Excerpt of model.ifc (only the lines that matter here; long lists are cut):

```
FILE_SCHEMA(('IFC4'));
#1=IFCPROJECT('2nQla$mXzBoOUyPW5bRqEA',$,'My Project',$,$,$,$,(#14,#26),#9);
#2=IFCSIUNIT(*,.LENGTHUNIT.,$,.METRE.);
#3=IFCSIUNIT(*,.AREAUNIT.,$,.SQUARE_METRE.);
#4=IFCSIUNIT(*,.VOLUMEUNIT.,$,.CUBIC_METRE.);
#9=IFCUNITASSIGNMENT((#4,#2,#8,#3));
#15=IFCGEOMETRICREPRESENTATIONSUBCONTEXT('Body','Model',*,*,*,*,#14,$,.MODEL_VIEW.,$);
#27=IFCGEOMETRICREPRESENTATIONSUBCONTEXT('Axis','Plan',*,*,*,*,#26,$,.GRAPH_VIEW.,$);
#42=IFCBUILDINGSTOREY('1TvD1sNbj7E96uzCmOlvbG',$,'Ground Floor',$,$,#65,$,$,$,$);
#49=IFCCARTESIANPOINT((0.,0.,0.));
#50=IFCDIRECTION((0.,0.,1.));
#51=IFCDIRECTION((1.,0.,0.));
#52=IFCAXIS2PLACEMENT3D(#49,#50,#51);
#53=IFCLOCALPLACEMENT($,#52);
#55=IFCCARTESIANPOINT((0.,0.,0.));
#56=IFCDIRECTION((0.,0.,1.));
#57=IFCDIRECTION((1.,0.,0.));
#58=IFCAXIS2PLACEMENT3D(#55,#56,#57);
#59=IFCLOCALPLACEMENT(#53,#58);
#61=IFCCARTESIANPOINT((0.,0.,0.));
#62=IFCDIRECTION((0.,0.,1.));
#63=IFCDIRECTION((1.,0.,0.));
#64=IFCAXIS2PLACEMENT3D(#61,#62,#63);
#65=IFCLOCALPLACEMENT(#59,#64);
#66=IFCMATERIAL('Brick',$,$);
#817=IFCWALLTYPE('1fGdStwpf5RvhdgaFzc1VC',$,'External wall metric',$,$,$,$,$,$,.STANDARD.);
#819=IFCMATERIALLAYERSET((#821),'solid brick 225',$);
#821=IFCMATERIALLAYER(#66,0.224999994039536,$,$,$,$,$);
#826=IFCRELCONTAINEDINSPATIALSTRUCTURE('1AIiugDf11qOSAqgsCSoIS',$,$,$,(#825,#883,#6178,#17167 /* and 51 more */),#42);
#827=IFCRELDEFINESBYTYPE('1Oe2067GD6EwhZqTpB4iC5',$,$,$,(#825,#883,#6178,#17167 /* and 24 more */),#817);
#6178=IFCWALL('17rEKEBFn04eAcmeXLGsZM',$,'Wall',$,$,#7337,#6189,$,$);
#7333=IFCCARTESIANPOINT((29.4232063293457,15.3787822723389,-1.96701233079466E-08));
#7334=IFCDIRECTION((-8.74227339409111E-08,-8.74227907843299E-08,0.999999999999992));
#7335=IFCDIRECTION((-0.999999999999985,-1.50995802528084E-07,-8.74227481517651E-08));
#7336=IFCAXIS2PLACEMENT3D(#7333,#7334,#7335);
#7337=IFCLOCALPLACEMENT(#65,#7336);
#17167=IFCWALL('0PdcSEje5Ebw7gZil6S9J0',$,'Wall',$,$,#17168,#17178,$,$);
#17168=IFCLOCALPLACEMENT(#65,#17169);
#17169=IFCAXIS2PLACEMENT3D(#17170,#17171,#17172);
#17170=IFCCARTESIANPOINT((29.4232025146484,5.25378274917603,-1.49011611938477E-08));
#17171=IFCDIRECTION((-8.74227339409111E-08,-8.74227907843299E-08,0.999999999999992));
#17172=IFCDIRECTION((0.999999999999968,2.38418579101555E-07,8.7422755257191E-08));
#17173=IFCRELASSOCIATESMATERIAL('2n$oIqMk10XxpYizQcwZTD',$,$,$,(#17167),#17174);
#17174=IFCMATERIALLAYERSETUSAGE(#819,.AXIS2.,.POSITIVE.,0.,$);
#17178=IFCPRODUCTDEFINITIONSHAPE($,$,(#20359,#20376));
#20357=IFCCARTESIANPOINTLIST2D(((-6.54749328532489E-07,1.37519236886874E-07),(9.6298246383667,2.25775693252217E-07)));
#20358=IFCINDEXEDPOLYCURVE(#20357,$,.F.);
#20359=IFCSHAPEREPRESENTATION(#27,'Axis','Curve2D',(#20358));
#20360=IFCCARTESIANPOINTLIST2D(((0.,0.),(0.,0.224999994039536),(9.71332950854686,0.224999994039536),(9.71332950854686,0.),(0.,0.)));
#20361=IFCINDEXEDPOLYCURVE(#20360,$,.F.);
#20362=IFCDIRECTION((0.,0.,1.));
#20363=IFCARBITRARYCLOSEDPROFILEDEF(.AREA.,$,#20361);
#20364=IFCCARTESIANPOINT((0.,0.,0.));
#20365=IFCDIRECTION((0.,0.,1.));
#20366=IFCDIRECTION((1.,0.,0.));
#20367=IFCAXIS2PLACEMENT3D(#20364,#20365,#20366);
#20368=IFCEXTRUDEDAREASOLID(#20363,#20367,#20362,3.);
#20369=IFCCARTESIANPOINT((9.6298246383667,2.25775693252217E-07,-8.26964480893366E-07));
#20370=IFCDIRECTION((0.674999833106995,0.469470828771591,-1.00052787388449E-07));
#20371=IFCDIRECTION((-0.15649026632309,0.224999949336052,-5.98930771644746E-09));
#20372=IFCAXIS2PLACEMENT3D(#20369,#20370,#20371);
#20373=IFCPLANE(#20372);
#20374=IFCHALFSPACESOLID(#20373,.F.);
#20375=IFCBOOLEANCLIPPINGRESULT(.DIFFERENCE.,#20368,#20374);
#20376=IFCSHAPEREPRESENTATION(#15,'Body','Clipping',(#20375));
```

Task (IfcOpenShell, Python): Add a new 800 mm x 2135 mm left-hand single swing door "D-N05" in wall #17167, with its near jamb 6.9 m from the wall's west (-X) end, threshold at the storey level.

```python
import numpy as np
import ifcopenshell
import ifcopenshell.api.feature
import ifcopenshell.api.geometry
import ifcopenshell.api.root
import ifcopenshell.api.spatial
import ifcopenshell.geom
import ifcopenshell.util.element
import ifcopenshell.util.placement
import ifcopenshell.util.representation
import ifcopenshell.util.shape
import ifcopenshell.util.unit

model = ifcopenshell.open("model.ifc")
unit_scale = ifcopenshell.util.unit.calculate_unit_scale(model)
settings = ifcopenshell.geom.settings()


def volume(element):
    """Net volume in cubic metres, openings subtracted."""
    shape = ifcopenshell.geom.create_shape(settings, element)
    return ifcopenshell.util.shape.get_volume(shape.geometry)


wall = model.by_guid("0PdcSEje5Ebw7gZil6S9J0")
storey = ifcopenshell.util.element.get_container(wall, ifc_class="IfcBuildingStorey")
context = ifcopenshell.util.representation.get_context(model, "Model", "Body", "MODEL_VIEW")
before = volume(wall)

width, height, from_end, sill = 0.8, 2.135, 6.9, 0.0  # metres

# The wall runs along its own X axis, and the end named is its -X end.
wall_shape = ifcopenshell.geom.create_shape(settings, wall)
x, y, z = ifcopenshell.util.shape.get_vertices(wall_shape.geometry).T
start = x.min() + from_end
face, thickness = float(y.min()), float(y.max() - y.min())
wall_matrix = ifcopenshell.util.placement.get_local_placement(wall.ObjectPlacement)
level = ifcopenshell.util.placement.get_local_placement(storey.ObjectPlacement)[2, 3]


def in_wall(x, y):
    """Placement at x, y metres in the wall's axes, at sill height."""
    matrix = wall_matrix.copy()
    matrix[:, 3] = wall_matrix @ np.array([x / unit_scale, y / unit_scale, 0.0, 1.0])
    matrix[2, 3] = level + sill / unit_scale
    return matrix


# Opening: a box that overshoots both wall faces by 50 mm.
opening = ifcopenshell.api.root.create_entity(model, ifc_class="IfcOpeningElement", predefined_type="OPENING")
box = ifcopenshell.api.geometry.add_wall_representation(
    model, context=context, length=width, height=height, thickness=thickness + 0.1
)
ifcopenshell.api.geometry.assign_representation(model, product=opening, representation=box)
ifcopenshell.api.geometry.edit_object_placement(model, product=opening, matrix=in_wall(start, face - 0.05), is_si=False)
ifcopenshell.api.feature.add_feature(model, feature=opening, element=wall)

door = ifcopenshell.api.root.create_entity(model, ifc_class="IfcDoor", name="D-N05", predefined_type="DOOR")
door.OverallWidth, door.OverallHeight = width / unit_scale, height / unit_scale
door.OperationType = "SINGLE_SWING_LEFT"
body = ifcopenshell.api.geometry.add_door_representation(
    model,
    context=context,
    overall_width=door.OverallWidth,
    overall_height=door.OverallHeight,
    operation_type="SINGLE_SWING_LEFT",
    lining_properties={"LiningDepth": thickness / unit_scale, "ThresholdDepth": thickness / unit_scale},
)
ifcopenshell.api.geometry.assign_representation(model, product=door, representation=body)
ifcopenshell.api.spatial.assign_container(model, products=[door], relating_structure=storey)
ifcopenshell.api.feature.add_filling(model, opening=opening, element=door)

# The lining spans the wall, so the door starts at the wall face.
ifcopenshell.api.geometry.edit_object_placement(model, product=door, matrix=in_wall(start, face), is_si=False)

after = volume(wall)

print(f"wall volume {before:.3f} -> {after:.3f} m3")

model.write("model-out.ifc")
```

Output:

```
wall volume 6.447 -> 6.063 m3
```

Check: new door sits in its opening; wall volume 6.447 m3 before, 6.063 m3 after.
